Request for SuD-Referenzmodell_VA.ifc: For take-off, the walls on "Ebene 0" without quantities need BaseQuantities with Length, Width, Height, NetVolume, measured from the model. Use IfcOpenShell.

First a look at what the model holds.

```python
import ifcopenshell
import ifcopenshell.util.element
import ifcopenshell.util.unit

model = ifcopenshell.open("SuD-Referenzmodell_VA.ifc")
print(model.schema)
for unit_type in ("LENGTHUNIT", "AREAUNIT", "VOLUMEUNIT"):
    print(unit_type, ifcopenshell.util.unit.calculate_unit_scale(model, unit_type))
storey = next(s for s in model.by_type("IfcBuildingStorey") if s.Name == "Ebene 0")
walls = [e for e in ifcopenshell.util.element.get_decomposition(storey) if e.is_a("IfcWall")]
for e in sorted(walls, key=lambda e: e.id()):
    print(e.id(), e.is_a(), e.Name, list(ifcopenshell.util.element.get_psets(e, qtos_only=True)), sep=" | ")
```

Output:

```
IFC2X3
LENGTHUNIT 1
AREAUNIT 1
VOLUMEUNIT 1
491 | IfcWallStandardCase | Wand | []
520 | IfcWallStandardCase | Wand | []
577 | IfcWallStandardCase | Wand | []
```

```python
import ifcopenshell
import ifcopenshell.api.pset
import ifcopenshell.geom
import ifcopenshell.util.element
import ifcopenshell.util.shape
import ifcopenshell.util.unit

model = ifcopenshell.open("SuD-Referenzmodell_VA.ifc")
unit_scale = ifcopenshell.util.unit.calculate_unit_scale(model)
volume_scale = ifcopenshell.util.unit.calculate_unit_scale(model, "VOLUMEUNIT")
settings = ifcopenshell.geom.settings()

storey = next(s for s in model.by_type("IfcBuildingStorey") if s.Name == "Ebene 0")
walls = [e for e in ifcopenshell.util.element.get_decomposition(storey) if e.is_a("IfcWall")]

for e in sorted(walls, key=lambda e: e.id()):
    if ifcopenshell.util.element.get_psets(e, qtos_only=True, should_inherit=False):
        continue
    # Geometry comes back in metres, in the element's own axes.
    shape = ifcopenshell.geom.create_shape(settings, e)
    values = {
        "Length": ifcopenshell.util.shape.get_x(shape.geometry) / unit_scale,
        "Width": ifcopenshell.util.shape.get_y(shape.geometry) / unit_scale,
        "Height": ifcopenshell.util.shape.get_z(shape.geometry) / unit_scale,
        "NetVolume": ifcopenshell.util.shape.get_volume(shape.geometry) / volume_scale,
    }
    qto = ifcopenshell.api.pset.add_qto(model, product=e, name="BaseQuantities")
    ifcopenshell.api.pset.edit_qto(model, qto=qto, properties=values)
    print(e.id(), {k: round(v, 3) for k, v in values.items()})

model.write("SuD-Referenzmodell_VA_updated.ifc")
```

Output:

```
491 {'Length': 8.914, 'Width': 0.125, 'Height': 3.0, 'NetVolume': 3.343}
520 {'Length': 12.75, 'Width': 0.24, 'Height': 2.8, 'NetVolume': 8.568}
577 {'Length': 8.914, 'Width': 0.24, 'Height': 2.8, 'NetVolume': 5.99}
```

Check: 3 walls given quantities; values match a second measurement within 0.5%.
